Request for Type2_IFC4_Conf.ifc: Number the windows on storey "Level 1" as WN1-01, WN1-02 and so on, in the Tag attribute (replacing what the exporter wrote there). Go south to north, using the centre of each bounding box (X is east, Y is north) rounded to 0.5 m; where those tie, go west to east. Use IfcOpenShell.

First a look at what the model holds.

```python
import ifcopenshell
import ifcopenshell.util.element
import ifcopenshell.util.placement

model = ifcopenshell.open("Type2_IFC4_Conf.ifc")
print(model.schema)
storey = next(s for s in model.by_type("IfcBuildingStorey") if s.Name == "Level 1")
windows = [e for e in ifcopenshell.util.element.get_decomposition(storey) if e.is_a("IfcWindow")]
for e in sorted(windows, key=lambda e: e.id()):
    origin = ifcopenshell.util.placement.get_local_placement(e.ObjectPlacement)[:3, 3]
    print(e.id(), e.Tag, e.Name, origin.round(2) + 0.0, sep=" | ")
```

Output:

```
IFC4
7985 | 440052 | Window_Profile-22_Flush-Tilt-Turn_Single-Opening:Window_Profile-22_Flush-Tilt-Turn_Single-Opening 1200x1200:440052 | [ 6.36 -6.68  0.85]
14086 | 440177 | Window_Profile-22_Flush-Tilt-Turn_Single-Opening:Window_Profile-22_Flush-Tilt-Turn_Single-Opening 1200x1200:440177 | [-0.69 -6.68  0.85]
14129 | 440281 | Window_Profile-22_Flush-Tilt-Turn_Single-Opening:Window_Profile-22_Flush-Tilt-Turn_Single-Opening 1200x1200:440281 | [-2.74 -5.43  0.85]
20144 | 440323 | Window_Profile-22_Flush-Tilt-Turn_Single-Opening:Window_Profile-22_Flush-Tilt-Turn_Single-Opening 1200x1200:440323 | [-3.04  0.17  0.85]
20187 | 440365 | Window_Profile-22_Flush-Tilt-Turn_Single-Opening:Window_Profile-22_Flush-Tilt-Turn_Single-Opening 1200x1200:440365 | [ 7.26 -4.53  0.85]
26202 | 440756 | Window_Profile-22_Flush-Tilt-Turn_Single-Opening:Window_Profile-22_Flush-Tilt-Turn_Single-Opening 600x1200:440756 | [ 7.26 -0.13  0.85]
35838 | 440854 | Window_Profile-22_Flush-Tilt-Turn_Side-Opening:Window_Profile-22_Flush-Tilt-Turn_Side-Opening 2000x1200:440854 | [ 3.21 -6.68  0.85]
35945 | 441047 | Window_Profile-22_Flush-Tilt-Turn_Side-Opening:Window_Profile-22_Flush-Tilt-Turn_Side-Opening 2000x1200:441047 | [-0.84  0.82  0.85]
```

```python
import ifcopenshell
import ifcopenshell.geom
import ifcopenshell.util.element
import ifcopenshell.util.shape

model = ifcopenshell.open("Type2_IFC4_Conf.ifc")
settings = ifcopenshell.geom.settings()
settings.set("use-world-coords", True)


def centre(element):
    shape = ifcopenshell.geom.create_shape(settings, element)
    return ifcopenshell.util.shape.get_bbox_centroid(shape.geometry)


storey = next(s for s in model.by_type("IfcBuildingStorey") if s.Name == "Level 1")
windows = [e for e in ifcopenshell.util.element.get_decomposition(storey) if e.is_a("IfcWindow")]

# Insertion points can sit at a corner or the storey origin, so sort by the geometry (in metres).
centres = {e: centre(e) for e in windows}
windows.sort(key=lambda e: (round(centres[e][1] / 0.5), centres[e][0]))

for i, e in enumerate(windows, start=1):
    number = f"WN1-{i:02d}"
    e.Tag = number
    print(e.id(), number)

model.write("Type2_IFC4_Conf_edited.ifc")
```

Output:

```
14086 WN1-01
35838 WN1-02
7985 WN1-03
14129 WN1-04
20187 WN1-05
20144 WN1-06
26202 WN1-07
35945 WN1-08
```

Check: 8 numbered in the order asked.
